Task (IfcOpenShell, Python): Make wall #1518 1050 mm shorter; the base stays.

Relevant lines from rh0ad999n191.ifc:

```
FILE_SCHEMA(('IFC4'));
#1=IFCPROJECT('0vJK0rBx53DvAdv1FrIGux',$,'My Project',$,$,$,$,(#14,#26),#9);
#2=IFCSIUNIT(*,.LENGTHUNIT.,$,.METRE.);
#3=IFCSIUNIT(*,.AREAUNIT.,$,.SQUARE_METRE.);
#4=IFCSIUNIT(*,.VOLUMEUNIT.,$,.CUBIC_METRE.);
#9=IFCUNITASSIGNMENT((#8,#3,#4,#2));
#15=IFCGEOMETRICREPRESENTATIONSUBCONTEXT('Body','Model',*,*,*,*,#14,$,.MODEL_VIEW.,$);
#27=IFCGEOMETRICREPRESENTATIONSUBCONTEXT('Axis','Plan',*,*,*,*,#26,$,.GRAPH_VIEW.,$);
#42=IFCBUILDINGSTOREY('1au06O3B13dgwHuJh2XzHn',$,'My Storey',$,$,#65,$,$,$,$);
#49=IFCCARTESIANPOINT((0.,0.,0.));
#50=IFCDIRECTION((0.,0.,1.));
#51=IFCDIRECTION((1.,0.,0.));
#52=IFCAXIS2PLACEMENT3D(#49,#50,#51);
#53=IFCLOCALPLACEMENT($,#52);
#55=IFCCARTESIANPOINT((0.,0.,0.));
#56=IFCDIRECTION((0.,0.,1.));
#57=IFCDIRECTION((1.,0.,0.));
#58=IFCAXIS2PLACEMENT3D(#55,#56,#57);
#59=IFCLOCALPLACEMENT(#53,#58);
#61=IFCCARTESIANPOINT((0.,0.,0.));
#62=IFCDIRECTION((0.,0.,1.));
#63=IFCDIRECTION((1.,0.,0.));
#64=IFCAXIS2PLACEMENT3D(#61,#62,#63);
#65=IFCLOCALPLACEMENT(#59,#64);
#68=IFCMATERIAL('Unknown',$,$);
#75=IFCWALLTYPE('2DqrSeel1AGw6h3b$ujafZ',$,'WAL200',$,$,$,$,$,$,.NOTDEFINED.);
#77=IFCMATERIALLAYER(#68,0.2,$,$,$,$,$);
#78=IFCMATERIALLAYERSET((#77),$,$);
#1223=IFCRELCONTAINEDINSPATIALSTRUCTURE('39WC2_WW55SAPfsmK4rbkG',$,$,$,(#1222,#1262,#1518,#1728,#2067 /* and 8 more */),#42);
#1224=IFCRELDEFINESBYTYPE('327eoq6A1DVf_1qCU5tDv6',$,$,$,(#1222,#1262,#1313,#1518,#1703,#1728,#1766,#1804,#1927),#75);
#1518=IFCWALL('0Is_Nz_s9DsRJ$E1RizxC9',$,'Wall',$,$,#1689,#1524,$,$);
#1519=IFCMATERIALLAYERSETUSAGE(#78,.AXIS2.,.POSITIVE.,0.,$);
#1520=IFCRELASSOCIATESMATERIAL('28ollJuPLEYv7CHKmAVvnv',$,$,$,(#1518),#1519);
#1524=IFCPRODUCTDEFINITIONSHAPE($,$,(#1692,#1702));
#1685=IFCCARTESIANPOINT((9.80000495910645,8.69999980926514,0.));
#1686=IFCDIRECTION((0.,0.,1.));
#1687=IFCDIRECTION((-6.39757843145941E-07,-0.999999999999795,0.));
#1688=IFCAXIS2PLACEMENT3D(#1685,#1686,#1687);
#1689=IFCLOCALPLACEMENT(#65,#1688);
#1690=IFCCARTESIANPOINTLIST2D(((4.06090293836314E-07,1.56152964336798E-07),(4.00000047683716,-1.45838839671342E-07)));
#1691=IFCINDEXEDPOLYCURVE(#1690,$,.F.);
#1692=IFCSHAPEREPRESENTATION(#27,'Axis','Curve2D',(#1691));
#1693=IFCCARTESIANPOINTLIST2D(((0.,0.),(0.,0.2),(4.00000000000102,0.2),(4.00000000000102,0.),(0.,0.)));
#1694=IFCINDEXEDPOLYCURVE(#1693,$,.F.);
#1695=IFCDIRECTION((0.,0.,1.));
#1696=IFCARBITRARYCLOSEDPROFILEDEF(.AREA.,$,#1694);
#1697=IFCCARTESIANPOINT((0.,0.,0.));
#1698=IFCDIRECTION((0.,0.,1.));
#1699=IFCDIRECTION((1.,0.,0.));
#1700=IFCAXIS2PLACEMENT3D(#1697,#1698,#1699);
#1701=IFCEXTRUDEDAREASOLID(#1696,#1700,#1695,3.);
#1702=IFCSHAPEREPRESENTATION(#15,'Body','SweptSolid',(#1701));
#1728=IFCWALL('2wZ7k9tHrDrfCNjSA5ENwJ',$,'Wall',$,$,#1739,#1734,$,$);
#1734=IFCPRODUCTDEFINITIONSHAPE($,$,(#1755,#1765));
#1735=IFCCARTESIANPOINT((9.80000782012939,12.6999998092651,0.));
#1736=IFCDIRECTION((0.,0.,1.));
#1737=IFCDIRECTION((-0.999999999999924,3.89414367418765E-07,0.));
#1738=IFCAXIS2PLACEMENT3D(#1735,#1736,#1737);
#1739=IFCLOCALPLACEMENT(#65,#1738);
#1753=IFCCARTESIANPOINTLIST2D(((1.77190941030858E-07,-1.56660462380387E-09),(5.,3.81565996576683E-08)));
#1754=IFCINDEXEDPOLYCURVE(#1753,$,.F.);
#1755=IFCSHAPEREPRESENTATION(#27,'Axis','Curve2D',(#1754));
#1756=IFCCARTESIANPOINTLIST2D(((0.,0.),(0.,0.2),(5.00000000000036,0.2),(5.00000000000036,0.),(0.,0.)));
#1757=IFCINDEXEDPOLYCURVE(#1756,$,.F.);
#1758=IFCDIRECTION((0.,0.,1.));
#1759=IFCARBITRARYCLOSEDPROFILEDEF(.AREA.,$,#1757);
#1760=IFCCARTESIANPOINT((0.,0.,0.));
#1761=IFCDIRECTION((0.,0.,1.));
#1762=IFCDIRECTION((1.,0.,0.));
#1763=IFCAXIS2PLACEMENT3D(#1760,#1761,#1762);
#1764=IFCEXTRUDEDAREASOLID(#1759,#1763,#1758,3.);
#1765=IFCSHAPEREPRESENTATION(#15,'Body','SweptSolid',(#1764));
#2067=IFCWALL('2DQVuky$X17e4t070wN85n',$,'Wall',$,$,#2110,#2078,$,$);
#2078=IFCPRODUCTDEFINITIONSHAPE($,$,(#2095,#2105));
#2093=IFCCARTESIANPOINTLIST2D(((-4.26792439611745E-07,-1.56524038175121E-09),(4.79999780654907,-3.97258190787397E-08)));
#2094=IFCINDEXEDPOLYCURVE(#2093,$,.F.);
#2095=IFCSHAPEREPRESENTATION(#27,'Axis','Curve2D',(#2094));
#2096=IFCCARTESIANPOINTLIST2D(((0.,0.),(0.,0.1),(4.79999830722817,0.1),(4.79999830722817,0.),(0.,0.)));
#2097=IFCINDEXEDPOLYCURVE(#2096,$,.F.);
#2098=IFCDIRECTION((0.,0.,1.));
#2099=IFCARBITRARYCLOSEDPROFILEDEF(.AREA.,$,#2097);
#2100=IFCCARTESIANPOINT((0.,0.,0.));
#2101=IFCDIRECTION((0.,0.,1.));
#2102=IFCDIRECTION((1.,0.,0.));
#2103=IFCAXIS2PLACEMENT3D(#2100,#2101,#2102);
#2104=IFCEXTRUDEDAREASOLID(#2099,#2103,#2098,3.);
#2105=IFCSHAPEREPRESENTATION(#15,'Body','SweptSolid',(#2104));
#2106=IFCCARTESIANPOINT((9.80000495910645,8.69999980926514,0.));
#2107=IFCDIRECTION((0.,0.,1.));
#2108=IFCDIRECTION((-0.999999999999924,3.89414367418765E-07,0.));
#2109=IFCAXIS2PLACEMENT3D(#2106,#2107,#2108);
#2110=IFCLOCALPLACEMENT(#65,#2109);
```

```python
import ifcopenshell
import ifcopenshell.geom
import ifcopenshell.util.representation
import ifcopenshell.util.shape

model = ifcopenshell.open("rh0ad999n191.ifc")
settings = ifcopenshell.geom.settings()


def volume(element):
    """Net volume in cubic metres, openings subtracted."""
    shape = ifcopenshell.geom.create_shape(settings, element)
    return ifcopenshell.util.shape.get_volume(shape.geometry)


wall = model.by_id(1518)
before = volume(wall)

body = ifcopenshell.util.representation.get_representation(wall, "Model", "Body")
solid = body.Items[0]
old_height = solid.Depth
solid.Depth -= 1.05
after = volume(wall)

print(f"height {old_height:g} -> {solid.Depth:g}, volume {before:.3f} -> {after:.3f} m3")

model.write("rh0ad999n191_v2.ifc")
```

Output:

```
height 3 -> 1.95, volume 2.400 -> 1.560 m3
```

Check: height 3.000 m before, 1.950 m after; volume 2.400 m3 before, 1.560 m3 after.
